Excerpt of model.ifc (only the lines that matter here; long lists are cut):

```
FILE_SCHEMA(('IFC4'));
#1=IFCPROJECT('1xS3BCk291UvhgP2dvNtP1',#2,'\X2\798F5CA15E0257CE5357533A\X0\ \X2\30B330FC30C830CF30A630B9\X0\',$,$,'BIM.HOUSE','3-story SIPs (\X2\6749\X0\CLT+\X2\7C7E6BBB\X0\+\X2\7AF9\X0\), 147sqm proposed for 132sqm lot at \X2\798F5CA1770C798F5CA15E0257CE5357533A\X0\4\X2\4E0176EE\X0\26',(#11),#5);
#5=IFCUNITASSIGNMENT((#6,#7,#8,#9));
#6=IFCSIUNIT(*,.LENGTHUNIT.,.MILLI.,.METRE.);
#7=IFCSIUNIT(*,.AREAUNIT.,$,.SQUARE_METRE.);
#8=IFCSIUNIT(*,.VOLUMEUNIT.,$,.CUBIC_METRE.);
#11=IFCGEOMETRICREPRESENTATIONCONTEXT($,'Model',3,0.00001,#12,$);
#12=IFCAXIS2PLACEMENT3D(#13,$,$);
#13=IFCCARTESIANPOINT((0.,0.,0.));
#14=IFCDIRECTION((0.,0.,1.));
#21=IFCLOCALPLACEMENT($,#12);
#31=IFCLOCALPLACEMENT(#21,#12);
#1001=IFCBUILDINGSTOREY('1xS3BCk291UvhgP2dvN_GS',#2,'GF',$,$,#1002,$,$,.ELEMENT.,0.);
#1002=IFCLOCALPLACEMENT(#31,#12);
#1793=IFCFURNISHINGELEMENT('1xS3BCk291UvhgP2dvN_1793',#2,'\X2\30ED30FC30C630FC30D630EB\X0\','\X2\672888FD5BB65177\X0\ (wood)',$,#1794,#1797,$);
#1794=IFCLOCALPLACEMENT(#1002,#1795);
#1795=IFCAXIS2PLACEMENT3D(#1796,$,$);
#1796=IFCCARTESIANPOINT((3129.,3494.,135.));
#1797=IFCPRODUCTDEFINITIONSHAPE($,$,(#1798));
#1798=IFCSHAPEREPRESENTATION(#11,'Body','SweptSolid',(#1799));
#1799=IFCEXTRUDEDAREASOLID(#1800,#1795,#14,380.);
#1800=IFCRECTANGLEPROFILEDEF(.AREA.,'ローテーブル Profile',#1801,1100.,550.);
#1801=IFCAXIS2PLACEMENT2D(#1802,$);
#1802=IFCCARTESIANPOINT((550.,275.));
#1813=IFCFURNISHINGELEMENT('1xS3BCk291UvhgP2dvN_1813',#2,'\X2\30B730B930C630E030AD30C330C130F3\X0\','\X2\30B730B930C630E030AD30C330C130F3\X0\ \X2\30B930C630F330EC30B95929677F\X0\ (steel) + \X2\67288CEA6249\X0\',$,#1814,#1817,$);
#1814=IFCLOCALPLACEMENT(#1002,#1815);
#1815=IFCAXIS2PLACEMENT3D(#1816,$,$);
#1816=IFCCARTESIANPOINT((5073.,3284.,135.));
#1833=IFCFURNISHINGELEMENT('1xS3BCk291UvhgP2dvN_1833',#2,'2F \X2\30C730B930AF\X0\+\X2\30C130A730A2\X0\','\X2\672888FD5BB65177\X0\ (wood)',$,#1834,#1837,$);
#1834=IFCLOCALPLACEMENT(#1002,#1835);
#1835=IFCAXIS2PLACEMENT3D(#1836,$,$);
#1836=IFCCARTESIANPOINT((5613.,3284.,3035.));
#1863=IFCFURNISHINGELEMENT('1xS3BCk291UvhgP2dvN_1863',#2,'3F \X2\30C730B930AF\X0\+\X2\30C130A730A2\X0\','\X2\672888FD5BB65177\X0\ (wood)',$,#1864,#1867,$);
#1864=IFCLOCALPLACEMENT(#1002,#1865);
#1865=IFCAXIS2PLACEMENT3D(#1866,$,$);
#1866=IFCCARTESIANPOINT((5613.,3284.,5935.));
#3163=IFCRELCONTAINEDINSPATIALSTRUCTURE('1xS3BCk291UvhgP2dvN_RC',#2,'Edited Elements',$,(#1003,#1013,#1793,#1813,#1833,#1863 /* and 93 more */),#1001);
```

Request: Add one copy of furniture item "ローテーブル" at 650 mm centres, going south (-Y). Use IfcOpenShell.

```python
import numpy as np
import ifcopenshell
import ifcopenshell.api.geometry
import ifcopenshell.api.root
import ifcopenshell.util.element
import ifcopenshell.util.placement
import ifcopenshell.util.unit

model = ifcopenshell.open("model.ifc")
unit_scale = ifcopenshell.util.unit.calculate_unit_scale(model)


def reuse_history(source, copy):
    """copy_class also copies each property set's owner history, people and application; keep the originals."""
    for rel in copy.IsDefinedBy:
        if rel.is_a("IfcRelDefinesByProperties") and (history := rel.RelatingPropertyDefinition.OwnerHistory):
            rel.RelatingPropertyDefinition.OwnerHistory = source.OwnerHistory
            ifcopenshell.util.element.remove_deep2(model, history)


source = model.by_guid("1xS3BCk291UvhgP2dvN_1793")
base = ifcopenshell.util.placement.get_local_placement(source.ObjectPlacement)
step = np.array([0.0, -1.0, 0.0]) * 0.65 / unit_scale

for i in range(1, 2):
    copy = ifcopenshell.api.root.copy_class(model, product=source)
    copy.Representation = ifcopenshell.util.element.copy_deep(
        model, source.Representation, exclude=["IfcGeometricRepresentationContext", "IfcRepresentationMap"]
    )
    reuse_history(source, copy)
    matrix = base.copy()
    matrix[:3, 3] += i * step
    print("added at", matrix[:3, 3].round(3) + 0.0)
    ifcopenshell.api.geometry.edit_object_placement(model, product=copy, matrix=matrix, is_si=False)

model.write("model_edited.ifc")
```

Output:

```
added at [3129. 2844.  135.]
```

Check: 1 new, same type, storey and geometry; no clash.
